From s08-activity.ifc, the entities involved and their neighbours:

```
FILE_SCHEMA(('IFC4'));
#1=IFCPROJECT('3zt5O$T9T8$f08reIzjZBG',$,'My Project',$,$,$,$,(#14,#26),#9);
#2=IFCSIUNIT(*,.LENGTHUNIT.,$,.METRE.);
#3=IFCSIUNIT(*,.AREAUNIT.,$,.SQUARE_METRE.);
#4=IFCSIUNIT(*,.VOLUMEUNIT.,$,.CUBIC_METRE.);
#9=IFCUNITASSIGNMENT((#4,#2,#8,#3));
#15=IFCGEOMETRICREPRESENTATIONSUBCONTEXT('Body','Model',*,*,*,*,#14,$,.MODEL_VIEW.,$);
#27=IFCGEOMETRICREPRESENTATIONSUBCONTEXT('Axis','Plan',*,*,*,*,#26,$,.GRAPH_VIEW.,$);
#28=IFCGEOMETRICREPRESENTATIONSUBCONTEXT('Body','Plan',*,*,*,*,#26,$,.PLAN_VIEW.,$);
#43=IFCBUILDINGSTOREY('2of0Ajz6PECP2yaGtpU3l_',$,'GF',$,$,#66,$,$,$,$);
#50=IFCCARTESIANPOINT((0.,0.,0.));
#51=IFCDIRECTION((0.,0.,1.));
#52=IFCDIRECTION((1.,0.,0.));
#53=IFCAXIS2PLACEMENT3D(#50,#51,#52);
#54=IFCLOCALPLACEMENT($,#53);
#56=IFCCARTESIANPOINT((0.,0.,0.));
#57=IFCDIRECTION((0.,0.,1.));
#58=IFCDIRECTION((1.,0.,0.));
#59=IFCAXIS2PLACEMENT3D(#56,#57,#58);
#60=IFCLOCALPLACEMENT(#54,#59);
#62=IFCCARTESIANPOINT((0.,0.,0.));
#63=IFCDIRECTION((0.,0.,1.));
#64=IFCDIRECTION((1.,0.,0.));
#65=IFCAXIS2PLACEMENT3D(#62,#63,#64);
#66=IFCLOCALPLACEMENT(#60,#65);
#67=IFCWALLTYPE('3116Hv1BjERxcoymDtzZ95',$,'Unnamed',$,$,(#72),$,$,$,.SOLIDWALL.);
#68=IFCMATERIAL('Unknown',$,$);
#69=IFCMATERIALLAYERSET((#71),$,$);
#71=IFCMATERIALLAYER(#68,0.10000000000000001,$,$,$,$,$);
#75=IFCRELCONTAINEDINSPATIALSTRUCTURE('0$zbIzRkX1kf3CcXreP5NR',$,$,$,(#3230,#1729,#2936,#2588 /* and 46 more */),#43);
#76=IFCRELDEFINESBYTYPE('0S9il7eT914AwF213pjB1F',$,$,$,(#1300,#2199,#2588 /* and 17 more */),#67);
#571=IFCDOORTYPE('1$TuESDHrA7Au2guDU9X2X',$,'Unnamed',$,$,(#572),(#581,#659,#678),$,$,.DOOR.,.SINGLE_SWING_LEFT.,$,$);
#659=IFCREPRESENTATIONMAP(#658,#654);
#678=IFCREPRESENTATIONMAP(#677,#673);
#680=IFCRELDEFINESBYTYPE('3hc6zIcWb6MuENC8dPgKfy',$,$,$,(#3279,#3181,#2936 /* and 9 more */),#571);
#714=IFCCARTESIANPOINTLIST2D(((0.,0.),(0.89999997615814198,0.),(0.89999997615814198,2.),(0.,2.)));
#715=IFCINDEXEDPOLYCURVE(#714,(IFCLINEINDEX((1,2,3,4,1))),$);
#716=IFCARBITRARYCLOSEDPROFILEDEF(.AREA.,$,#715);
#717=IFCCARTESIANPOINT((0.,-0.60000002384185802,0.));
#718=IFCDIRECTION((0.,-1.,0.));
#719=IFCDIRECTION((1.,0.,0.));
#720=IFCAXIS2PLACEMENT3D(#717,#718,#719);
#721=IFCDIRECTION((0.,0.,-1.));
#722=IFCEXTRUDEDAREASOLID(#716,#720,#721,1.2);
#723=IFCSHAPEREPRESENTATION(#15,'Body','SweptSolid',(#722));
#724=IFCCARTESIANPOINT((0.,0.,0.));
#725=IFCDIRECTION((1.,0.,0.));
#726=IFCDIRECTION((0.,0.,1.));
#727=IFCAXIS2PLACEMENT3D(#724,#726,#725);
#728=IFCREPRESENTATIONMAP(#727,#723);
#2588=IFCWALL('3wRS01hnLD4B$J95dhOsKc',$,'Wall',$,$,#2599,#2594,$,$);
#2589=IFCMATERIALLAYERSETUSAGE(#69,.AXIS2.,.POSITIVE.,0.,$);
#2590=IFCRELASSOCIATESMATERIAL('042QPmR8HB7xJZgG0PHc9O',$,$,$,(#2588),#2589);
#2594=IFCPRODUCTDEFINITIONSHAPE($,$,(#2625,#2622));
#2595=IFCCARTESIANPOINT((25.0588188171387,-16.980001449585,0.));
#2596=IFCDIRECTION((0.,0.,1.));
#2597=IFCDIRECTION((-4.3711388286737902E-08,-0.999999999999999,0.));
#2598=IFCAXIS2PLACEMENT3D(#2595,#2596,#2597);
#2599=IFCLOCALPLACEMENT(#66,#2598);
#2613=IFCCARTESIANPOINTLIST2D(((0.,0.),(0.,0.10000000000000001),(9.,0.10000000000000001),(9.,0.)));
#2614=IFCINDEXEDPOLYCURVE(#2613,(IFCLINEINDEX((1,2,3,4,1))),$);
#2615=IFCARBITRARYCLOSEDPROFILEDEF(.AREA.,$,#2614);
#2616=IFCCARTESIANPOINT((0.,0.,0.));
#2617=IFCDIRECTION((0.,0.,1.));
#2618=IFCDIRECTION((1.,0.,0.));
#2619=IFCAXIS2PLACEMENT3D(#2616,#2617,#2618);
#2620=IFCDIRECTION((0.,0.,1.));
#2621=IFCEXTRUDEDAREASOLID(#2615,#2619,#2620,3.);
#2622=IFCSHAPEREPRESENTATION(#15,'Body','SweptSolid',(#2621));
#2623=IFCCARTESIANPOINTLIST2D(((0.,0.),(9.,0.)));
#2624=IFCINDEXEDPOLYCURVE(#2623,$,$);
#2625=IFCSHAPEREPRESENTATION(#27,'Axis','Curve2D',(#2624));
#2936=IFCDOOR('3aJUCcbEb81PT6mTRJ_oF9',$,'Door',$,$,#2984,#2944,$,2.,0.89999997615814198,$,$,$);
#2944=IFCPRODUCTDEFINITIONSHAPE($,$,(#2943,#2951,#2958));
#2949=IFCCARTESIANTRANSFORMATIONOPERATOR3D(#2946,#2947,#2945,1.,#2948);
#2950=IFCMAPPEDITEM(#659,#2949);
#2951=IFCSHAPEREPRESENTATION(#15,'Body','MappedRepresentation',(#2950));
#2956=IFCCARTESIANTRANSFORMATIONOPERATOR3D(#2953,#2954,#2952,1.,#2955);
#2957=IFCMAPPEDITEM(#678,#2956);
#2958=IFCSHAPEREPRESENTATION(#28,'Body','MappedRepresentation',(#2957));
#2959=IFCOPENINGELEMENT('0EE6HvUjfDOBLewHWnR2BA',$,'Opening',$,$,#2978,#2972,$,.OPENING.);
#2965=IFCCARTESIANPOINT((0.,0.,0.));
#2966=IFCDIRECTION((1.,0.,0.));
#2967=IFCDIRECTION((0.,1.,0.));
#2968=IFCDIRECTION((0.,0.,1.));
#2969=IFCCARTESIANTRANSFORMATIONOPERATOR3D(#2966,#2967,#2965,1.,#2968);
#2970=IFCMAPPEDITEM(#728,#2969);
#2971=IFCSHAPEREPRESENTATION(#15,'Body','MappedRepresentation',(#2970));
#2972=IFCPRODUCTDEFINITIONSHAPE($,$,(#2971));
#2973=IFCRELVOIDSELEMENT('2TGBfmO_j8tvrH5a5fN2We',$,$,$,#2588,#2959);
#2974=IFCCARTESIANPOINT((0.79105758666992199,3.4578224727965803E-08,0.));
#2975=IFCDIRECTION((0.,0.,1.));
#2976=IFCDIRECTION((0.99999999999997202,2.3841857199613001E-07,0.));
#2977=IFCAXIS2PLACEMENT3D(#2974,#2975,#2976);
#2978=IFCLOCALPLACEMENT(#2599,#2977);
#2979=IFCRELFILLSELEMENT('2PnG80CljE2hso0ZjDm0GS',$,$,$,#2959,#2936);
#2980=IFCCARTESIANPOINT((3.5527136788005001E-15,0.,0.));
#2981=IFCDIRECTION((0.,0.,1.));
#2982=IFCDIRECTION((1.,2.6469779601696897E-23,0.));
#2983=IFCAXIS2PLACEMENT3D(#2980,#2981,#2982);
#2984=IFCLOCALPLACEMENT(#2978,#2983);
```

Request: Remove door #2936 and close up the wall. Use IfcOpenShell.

```python
import ifcopenshell
import ifcopenshell.api.feature
import ifcopenshell.api.root
import ifcopenshell.geom
import ifcopenshell.util.shape

model = ifcopenshell.open("s08-activity.ifc")
settings = ifcopenshell.geom.settings()


def volume(element):
    """Net volume in cubic metres, openings subtracted."""
    shape = ifcopenshell.geom.create_shape(settings, element)
    return ifcopenshell.util.shape.get_volume(shape.geometry)


door = model.by_guid("3aJUCcbEb81PT6mTRJ_oF9")
opening = door.FillsVoids[0].RelatingOpeningElement
wall = opening.VoidsElements[0].RelatingBuildingElement
before = volume(wall)

ifcopenshell.api.root.remove_product(model, product=door)
ifcopenshell.api.feature.remove_feature(model, feature=opening)

after = volume(wall)

print(f"wall volume {before:.3f} -> {after:.3f} m3")

model.write("s08-activity-out.ifc")
```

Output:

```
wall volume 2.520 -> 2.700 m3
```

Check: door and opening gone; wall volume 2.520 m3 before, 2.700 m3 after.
